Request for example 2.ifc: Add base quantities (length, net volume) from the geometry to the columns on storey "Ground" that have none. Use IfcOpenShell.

First a look at what the model holds.

```python
import ifcopenshell
import ifcopenshell.util.element
import ifcopenshell.util.unit

model = ifcopenshell.open("example 2.ifc")
print(model.schema)
for unit_type in ("LENGTHUNIT", "AREAUNIT", "VOLUMEUNIT"):
    print(unit_type, ifcopenshell.util.unit.calculate_unit_scale(model, unit_type))
storey = next(s for s in model.by_type("IfcBuildingStorey") if s.Name == "Ground")
columns = [e for e in ifcopenshell.util.element.get_decomposition(storey) if e.is_a("IfcColumn")]
for e in sorted(columns, key=lambda e: e.id()):
    print(e.id(), e.is_a(), e.Name, list(ifcopenshell.util.element.get_psets(e, qtos_only=True)), sep=" | ")
```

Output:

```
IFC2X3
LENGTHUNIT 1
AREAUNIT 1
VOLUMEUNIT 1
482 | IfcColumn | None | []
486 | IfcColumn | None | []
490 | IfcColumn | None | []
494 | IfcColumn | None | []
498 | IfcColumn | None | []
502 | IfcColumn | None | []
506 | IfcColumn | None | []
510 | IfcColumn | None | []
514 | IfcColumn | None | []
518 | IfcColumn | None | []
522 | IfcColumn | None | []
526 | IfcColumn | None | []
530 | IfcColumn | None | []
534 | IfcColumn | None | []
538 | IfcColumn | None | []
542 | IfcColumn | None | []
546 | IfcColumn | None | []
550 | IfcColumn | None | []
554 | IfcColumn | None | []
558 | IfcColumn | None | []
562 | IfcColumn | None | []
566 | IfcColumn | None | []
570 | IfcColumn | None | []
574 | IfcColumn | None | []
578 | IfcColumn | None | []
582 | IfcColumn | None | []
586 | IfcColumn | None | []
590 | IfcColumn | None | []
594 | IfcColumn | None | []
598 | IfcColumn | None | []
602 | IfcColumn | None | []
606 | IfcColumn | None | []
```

```python
import ifcopenshell
import ifcopenshell.api.pset
import ifcopenshell.geom
import ifcopenshell.util.element
import ifcopenshell.util.shape
import ifcopenshell.util.unit

model = ifcopenshell.open("example 2.ifc")
unit_scale = ifcopenshell.util.unit.calculate_unit_scale(model)
volume_scale = ifcopenshell.util.unit.calculate_unit_scale(model, "VOLUMEUNIT")
settings = ifcopenshell.geom.settings()

storey = next(s for s in model.by_type("IfcBuildingStorey") if s.Name == "Ground")
columns = [e for e in ifcopenshell.util.element.get_decomposition(storey) if e.is_a("IfcColumn")]

for e in sorted(columns, key=lambda e: e.id()):
    if ifcopenshell.util.element.get_psets(e, qtos_only=True, should_inherit=False):
        continue
    # Geometry comes back in metres, in the element's own axes.
    shape = ifcopenshell.geom.create_shape(settings, e)
    values = {
        "Length": ifcopenshell.util.shape.get_z(shape.geometry) / unit_scale,
        "NetVolume": ifcopenshell.util.shape.get_volume(shape.geometry) / volume_scale,
    }
    qto = ifcopenshell.api.pset.add_qto(model, product=e, name="BaseQuantities")
    ifcopenshell.api.pset.edit_qto(model, qto=qto, properties=values)
    print(e.id(), {k: round(v, 3) for k, v in values.items()})

model.write("example 2_v2.ifc")
```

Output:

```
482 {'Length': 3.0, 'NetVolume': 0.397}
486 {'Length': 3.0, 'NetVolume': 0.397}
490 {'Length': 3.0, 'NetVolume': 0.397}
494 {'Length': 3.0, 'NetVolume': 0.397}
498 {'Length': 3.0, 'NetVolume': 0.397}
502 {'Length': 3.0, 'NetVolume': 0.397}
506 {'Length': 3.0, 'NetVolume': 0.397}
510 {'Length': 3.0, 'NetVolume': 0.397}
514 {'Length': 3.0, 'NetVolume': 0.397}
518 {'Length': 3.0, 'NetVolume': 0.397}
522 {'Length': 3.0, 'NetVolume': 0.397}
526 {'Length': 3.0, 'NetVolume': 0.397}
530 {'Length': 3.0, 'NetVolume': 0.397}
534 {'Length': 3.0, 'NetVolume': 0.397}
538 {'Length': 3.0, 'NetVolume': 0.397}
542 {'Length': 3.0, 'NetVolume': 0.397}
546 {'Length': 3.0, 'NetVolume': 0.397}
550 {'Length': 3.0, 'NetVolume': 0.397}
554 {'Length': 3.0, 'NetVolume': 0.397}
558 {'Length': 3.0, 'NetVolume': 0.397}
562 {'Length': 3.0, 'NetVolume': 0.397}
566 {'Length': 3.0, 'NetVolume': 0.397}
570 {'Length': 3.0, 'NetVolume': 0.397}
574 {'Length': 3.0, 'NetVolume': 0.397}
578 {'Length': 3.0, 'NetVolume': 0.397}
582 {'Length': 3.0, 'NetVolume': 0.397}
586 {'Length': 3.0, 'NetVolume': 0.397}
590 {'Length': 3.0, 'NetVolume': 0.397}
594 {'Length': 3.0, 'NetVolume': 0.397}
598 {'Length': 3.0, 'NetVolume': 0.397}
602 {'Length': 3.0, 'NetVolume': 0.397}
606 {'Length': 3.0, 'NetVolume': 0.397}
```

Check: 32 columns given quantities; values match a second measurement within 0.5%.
